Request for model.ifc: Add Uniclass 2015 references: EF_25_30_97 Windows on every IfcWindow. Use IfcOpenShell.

First a look at what the model holds.

```python
import ifcopenshell

model = ifcopenshell.open("model.ifc")
print(model.schema)
print("classifications:", [c.Name for c in model.by_type("IfcClassification")])
for ifc_class in ("IfcDoor", "IfcRoof", "IfcStair", "IfcWall", "IfcWindow"):
    print(ifc_class, len(model.by_type(ifc_class)))
```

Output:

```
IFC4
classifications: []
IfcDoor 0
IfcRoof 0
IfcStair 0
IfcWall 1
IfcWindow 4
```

```python
import ifcopenshell
import ifcopenshell.api.classification

model = ifcopenshell.open("model.ifc")

system = ifcopenshell.api.classification.add_classification(model, classification="Uniclass 2015")

codes = {
    "IfcWindow": ("EF_25_30_97", "Windows"),
}
for ifc_class, (code, name) in codes.items():
    products = model.by_type(ifc_class)
    ifcopenshell.api.classification.add_reference(
        model, products=products, classification=system, identification=code, name=name
    )
    print(code, len(products))

model.write("model_edited.ifc")
```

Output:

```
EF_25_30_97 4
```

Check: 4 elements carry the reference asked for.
